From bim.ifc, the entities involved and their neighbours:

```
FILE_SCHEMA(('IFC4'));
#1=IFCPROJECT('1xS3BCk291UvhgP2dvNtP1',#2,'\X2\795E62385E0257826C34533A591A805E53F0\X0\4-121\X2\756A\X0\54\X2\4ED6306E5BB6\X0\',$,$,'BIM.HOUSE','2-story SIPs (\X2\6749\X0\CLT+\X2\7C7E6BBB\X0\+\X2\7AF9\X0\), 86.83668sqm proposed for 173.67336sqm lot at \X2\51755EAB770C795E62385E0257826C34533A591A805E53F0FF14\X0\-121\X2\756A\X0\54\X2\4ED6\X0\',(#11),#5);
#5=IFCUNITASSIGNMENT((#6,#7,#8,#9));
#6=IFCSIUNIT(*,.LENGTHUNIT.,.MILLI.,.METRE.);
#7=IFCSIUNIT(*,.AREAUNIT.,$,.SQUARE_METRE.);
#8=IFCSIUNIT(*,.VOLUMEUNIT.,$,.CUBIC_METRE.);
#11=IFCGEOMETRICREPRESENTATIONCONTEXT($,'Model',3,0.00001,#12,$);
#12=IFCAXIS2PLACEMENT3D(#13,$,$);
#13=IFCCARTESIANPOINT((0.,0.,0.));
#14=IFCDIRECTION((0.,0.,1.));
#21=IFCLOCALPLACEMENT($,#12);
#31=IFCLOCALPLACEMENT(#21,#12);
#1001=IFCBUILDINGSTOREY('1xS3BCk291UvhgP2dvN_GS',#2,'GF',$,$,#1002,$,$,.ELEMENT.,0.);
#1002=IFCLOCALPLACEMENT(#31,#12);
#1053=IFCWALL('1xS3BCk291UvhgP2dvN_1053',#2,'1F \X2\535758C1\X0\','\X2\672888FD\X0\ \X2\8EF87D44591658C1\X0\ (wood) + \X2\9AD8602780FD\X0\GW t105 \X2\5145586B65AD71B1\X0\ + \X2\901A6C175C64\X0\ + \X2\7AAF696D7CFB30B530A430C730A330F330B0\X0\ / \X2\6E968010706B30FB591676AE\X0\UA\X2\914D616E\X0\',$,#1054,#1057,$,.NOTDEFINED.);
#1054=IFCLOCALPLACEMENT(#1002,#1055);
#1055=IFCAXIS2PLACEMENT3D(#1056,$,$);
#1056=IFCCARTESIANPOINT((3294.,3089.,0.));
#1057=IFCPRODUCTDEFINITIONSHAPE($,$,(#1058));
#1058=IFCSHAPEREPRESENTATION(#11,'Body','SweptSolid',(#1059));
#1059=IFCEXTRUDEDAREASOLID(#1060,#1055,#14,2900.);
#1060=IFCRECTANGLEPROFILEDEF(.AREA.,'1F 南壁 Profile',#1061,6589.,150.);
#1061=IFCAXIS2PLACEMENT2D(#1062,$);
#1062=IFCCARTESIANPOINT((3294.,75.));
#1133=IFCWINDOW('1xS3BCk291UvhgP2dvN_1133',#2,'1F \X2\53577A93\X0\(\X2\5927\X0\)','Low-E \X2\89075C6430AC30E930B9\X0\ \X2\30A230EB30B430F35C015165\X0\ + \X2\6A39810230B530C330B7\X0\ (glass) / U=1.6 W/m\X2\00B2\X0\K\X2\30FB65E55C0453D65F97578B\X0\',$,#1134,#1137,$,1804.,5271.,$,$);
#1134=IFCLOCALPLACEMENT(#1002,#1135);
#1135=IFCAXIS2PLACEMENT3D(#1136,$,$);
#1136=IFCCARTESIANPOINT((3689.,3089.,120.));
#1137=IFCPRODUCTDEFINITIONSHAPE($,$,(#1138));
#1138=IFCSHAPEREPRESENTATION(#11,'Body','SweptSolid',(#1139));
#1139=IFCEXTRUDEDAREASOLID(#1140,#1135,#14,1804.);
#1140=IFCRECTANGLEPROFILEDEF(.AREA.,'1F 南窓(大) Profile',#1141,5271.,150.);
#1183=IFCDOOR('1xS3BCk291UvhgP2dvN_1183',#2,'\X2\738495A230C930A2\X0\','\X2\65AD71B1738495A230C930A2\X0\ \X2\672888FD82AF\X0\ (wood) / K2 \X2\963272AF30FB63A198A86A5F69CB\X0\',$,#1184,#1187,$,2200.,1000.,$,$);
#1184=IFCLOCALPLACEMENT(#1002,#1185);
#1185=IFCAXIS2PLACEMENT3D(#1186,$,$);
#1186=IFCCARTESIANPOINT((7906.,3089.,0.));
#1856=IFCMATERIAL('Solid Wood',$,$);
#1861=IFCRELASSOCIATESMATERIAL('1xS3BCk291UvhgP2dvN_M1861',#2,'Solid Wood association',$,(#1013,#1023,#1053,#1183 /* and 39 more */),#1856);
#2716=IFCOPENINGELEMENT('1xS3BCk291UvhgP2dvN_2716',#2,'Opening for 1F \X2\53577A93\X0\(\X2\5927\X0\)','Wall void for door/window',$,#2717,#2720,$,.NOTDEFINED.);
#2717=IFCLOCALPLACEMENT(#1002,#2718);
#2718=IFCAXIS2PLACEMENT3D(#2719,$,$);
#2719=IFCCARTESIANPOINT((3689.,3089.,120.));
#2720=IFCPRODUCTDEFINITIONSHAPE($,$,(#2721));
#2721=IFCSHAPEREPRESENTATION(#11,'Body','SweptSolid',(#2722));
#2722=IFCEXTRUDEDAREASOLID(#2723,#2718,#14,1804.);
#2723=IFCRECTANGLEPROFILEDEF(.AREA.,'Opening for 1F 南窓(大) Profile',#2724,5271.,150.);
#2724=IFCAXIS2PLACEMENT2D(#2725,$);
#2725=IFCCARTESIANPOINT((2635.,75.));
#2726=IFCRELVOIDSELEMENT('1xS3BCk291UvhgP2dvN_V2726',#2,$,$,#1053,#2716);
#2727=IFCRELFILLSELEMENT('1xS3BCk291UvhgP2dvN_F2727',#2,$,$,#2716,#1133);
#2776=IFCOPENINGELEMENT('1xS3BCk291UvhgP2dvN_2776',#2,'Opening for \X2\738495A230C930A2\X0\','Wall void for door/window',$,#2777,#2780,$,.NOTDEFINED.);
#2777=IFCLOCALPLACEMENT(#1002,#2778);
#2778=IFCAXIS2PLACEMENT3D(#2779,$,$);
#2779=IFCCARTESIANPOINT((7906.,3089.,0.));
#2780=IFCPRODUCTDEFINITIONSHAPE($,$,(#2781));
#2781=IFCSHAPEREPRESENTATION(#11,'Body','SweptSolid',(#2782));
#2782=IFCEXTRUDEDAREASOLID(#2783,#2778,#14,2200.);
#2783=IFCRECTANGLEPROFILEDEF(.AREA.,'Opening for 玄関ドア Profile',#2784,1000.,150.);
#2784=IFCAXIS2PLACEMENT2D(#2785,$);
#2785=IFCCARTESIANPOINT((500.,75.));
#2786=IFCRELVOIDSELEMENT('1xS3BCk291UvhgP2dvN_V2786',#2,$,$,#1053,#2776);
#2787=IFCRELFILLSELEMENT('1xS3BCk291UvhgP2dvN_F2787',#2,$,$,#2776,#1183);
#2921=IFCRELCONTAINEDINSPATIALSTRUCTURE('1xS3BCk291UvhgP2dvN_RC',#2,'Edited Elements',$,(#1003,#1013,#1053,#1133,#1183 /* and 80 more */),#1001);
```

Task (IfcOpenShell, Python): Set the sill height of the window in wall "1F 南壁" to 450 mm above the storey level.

```python
import numpy as np
import ifcopenshell
import ifcopenshell.api.geometry
import ifcopenshell.geom
import ifcopenshell.util.element
import ifcopenshell.util.placement
import ifcopenshell.util.shape
import ifcopenshell.util.unit

model = ifcopenshell.open("bim.ifc")
unit_scale = ifcopenshell.util.unit.calculate_unit_scale(model)

window = model.by_id(1133)
opening = window.FillsVoids[0].RelatingOpeningElement
storey = ifcopenshell.util.element.get_container(window, ifc_class="IfcBuildingStorey")
level = ifcopenshell.util.placement.get_local_placement(storey.ObjectPlacement)[2, 3]

# The opening's origin need not be at the sill, so measure its lowest point.
shape = ifcopenshell.geom.create_shape(ifcopenshell.geom.settings(), opening)
bottom = ifcopenshell.util.shape.get_shape_bottom_elevation(shape, shape.geometry) / unit_scale
dz = level + 0.45 / unit_scale - bottom

shift = np.array([0.0, 0.0, dz])
# The window is not placed relative to its opening, so move both.
for product in (opening, window):
    matrix = ifcopenshell.util.placement.get_local_placement(product.ObjectPlacement)
    matrix[:3, 3] += shift
    ifcopenshell.api.geometry.edit_object_placement(model, product=product, matrix=matrix, is_si=False)

print(f"moved by {dz * unit_scale:+.3f} m")

model.write("bim_edited.ifc")
```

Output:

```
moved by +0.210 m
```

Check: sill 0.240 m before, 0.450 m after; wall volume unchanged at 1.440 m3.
